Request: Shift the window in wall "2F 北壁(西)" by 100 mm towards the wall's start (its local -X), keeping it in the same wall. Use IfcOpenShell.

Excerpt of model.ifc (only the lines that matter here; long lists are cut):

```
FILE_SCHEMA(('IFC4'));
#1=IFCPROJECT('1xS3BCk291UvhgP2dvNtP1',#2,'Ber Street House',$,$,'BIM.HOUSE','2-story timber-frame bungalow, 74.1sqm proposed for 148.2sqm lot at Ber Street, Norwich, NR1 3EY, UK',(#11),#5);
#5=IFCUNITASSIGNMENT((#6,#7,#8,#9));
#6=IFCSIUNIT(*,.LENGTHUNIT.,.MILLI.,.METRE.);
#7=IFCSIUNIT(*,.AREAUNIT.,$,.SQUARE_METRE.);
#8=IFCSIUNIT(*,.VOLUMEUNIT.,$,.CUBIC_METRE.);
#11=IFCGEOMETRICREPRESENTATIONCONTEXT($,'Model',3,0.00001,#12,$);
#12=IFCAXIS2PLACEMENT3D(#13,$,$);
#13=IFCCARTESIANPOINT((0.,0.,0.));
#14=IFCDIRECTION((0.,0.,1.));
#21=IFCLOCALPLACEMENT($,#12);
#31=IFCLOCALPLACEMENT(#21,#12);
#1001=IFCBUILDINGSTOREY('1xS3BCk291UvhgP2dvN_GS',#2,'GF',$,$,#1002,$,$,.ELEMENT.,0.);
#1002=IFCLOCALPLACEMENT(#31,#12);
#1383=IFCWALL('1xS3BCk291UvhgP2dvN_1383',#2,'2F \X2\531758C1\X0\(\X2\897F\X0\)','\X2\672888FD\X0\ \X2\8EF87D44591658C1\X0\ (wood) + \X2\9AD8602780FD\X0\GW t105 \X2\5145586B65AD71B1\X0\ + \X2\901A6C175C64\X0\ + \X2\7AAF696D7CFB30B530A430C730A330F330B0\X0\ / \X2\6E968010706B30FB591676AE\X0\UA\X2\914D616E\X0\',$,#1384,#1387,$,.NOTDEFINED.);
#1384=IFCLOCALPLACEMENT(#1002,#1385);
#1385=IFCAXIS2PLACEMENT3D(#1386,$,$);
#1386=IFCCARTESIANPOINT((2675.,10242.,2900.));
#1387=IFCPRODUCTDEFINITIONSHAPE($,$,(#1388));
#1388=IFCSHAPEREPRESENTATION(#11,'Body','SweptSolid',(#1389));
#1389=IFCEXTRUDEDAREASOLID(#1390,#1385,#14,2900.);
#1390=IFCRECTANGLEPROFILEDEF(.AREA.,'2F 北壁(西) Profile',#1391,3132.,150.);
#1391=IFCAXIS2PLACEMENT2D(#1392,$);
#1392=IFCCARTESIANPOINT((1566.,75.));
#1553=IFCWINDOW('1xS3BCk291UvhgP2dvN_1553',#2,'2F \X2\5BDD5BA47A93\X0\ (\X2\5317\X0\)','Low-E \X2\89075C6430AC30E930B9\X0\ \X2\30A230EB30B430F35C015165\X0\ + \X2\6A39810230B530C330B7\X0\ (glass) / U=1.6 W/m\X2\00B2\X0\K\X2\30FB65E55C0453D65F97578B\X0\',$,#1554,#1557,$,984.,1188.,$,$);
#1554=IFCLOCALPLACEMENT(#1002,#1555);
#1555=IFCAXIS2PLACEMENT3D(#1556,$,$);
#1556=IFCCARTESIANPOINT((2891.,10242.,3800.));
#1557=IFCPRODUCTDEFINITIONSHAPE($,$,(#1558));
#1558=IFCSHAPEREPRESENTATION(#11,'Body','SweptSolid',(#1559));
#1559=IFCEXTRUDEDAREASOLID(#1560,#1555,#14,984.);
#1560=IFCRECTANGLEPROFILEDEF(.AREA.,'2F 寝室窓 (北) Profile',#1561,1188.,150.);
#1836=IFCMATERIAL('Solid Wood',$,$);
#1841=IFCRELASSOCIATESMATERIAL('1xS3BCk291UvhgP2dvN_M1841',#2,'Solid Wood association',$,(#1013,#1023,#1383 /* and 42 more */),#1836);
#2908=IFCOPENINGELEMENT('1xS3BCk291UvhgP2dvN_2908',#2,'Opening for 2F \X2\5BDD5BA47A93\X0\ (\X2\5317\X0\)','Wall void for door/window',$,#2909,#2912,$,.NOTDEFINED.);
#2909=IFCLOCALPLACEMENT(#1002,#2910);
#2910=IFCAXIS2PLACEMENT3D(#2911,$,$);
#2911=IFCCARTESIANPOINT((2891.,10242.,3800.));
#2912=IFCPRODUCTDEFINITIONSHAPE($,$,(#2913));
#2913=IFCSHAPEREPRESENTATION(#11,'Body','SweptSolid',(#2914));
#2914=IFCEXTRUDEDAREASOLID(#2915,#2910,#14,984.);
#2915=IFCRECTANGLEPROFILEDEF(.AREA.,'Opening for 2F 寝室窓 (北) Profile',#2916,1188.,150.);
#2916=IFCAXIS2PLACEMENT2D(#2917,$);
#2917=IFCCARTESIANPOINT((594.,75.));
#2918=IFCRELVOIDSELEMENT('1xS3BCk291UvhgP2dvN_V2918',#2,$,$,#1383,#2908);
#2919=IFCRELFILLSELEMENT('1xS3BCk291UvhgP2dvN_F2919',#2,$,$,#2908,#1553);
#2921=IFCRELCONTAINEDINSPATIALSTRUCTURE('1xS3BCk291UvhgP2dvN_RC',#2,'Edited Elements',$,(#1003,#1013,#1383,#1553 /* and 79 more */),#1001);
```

```python
import ifcopenshell
import ifcopenshell.api.geometry
import ifcopenshell.util.placement
import ifcopenshell.util.unit

model = ifcopenshell.open("model.ifc")
unit_scale = ifcopenshell.util.unit.calculate_unit_scale(model)

window = model.by_guid("1xS3BCk291UvhgP2dvN_1553")
opening = window.FillsVoids[0].RelatingOpeningElement
wall = opening.VoidsElements[0].RelatingBuildingElement

wall_matrix = ifcopenshell.util.placement.get_local_placement(wall.ObjectPlacement)
shift = wall_matrix[:3, 0] * -0.1 / unit_scale
before = ifcopenshell.util.placement.get_local_placement(window.ObjectPlacement)[:3, 3].copy()

# The window is not placed relative to its opening, so move both.
for product in (opening, window):
    matrix = ifcopenshell.util.placement.get_local_placement(product.ObjectPlacement)
    matrix[:3, 3] += shift
    ifcopenshell.api.geometry.edit_object_placement(model, product=product, matrix=matrix, is_si=False)

after = ifcopenshell.util.placement.get_local_placement(window.ObjectPlacement)[:3, 3]
print("window moved by", (after - before).round(3) + 0.0)

model.write("model-out.ifc")
```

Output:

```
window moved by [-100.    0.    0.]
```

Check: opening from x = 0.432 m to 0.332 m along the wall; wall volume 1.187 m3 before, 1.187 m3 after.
